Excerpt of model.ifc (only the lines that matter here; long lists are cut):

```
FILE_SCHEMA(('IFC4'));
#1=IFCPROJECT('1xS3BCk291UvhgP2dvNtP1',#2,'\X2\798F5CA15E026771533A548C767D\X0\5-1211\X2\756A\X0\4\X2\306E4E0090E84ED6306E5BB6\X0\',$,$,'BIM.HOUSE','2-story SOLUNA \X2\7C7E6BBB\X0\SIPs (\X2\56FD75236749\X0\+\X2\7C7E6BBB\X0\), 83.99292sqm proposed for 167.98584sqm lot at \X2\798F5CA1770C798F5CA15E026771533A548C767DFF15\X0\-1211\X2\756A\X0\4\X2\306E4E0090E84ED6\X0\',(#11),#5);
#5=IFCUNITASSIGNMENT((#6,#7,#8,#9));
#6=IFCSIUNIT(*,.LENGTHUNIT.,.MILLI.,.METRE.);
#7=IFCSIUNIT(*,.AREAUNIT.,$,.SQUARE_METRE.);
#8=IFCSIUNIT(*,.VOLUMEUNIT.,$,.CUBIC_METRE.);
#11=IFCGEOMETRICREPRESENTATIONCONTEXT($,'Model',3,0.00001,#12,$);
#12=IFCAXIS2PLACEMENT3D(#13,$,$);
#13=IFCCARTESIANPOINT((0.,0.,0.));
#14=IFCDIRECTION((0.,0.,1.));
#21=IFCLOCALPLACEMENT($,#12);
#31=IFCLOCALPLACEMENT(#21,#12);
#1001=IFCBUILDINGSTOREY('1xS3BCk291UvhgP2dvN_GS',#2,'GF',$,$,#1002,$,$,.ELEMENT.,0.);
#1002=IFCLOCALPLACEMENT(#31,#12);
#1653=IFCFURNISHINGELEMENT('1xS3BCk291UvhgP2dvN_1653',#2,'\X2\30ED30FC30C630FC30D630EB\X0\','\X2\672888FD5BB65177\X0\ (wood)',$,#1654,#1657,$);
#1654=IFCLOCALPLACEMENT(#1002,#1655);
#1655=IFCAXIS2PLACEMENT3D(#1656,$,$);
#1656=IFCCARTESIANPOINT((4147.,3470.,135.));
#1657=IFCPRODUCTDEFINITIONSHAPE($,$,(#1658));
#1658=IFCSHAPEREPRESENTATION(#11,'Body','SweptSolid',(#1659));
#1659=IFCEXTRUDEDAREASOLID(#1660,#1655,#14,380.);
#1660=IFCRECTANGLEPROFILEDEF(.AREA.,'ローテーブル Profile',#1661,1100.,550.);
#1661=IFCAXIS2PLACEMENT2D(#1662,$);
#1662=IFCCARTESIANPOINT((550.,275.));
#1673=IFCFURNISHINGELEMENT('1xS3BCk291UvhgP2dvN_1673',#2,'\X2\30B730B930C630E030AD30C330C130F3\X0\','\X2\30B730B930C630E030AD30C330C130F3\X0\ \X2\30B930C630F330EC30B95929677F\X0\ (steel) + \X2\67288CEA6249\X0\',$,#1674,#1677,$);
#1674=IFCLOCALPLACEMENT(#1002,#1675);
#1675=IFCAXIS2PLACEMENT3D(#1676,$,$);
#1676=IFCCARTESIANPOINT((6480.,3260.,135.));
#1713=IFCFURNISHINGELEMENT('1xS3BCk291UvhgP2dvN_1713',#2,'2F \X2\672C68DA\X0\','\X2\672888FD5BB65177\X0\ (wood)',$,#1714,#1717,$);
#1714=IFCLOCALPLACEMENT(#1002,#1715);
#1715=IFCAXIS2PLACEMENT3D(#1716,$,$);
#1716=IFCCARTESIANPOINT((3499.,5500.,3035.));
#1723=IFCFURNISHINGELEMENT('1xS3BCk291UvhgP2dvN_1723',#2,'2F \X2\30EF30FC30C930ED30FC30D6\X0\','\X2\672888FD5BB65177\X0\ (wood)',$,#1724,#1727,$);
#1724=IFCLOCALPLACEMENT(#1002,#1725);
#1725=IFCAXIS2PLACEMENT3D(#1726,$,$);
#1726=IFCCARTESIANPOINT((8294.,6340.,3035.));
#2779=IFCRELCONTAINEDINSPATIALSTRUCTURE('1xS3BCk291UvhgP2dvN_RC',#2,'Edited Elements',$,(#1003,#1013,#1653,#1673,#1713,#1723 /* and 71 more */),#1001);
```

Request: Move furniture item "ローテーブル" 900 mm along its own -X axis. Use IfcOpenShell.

```python
import ifcopenshell
import ifcopenshell.api.geometry
import ifcopenshell.util.placement
import ifcopenshell.util.unit

model = ifcopenshell.open("model.ifc")
unit_scale = ifcopenshell.util.unit.calculate_unit_scale(model)

item = model.by_id(1653)
matrix = ifcopenshell.util.placement.get_local_placement(item.ObjectPlacement)
matrix[:3, 3] -= matrix[:3, 0] * 0.9 / unit_scale
ifcopenshell.api.geometry.edit_object_placement(model, product=item, matrix=matrix, is_si=False)

print(ifcopenshell.util.placement.get_local_placement(item.ObjectPlacement).round(3) + 0.0)

model.write("model_updated.ifc")
```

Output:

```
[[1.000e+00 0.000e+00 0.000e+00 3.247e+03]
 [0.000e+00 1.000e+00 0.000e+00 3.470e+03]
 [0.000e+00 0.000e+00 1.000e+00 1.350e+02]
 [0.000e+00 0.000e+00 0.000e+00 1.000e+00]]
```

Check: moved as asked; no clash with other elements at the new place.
